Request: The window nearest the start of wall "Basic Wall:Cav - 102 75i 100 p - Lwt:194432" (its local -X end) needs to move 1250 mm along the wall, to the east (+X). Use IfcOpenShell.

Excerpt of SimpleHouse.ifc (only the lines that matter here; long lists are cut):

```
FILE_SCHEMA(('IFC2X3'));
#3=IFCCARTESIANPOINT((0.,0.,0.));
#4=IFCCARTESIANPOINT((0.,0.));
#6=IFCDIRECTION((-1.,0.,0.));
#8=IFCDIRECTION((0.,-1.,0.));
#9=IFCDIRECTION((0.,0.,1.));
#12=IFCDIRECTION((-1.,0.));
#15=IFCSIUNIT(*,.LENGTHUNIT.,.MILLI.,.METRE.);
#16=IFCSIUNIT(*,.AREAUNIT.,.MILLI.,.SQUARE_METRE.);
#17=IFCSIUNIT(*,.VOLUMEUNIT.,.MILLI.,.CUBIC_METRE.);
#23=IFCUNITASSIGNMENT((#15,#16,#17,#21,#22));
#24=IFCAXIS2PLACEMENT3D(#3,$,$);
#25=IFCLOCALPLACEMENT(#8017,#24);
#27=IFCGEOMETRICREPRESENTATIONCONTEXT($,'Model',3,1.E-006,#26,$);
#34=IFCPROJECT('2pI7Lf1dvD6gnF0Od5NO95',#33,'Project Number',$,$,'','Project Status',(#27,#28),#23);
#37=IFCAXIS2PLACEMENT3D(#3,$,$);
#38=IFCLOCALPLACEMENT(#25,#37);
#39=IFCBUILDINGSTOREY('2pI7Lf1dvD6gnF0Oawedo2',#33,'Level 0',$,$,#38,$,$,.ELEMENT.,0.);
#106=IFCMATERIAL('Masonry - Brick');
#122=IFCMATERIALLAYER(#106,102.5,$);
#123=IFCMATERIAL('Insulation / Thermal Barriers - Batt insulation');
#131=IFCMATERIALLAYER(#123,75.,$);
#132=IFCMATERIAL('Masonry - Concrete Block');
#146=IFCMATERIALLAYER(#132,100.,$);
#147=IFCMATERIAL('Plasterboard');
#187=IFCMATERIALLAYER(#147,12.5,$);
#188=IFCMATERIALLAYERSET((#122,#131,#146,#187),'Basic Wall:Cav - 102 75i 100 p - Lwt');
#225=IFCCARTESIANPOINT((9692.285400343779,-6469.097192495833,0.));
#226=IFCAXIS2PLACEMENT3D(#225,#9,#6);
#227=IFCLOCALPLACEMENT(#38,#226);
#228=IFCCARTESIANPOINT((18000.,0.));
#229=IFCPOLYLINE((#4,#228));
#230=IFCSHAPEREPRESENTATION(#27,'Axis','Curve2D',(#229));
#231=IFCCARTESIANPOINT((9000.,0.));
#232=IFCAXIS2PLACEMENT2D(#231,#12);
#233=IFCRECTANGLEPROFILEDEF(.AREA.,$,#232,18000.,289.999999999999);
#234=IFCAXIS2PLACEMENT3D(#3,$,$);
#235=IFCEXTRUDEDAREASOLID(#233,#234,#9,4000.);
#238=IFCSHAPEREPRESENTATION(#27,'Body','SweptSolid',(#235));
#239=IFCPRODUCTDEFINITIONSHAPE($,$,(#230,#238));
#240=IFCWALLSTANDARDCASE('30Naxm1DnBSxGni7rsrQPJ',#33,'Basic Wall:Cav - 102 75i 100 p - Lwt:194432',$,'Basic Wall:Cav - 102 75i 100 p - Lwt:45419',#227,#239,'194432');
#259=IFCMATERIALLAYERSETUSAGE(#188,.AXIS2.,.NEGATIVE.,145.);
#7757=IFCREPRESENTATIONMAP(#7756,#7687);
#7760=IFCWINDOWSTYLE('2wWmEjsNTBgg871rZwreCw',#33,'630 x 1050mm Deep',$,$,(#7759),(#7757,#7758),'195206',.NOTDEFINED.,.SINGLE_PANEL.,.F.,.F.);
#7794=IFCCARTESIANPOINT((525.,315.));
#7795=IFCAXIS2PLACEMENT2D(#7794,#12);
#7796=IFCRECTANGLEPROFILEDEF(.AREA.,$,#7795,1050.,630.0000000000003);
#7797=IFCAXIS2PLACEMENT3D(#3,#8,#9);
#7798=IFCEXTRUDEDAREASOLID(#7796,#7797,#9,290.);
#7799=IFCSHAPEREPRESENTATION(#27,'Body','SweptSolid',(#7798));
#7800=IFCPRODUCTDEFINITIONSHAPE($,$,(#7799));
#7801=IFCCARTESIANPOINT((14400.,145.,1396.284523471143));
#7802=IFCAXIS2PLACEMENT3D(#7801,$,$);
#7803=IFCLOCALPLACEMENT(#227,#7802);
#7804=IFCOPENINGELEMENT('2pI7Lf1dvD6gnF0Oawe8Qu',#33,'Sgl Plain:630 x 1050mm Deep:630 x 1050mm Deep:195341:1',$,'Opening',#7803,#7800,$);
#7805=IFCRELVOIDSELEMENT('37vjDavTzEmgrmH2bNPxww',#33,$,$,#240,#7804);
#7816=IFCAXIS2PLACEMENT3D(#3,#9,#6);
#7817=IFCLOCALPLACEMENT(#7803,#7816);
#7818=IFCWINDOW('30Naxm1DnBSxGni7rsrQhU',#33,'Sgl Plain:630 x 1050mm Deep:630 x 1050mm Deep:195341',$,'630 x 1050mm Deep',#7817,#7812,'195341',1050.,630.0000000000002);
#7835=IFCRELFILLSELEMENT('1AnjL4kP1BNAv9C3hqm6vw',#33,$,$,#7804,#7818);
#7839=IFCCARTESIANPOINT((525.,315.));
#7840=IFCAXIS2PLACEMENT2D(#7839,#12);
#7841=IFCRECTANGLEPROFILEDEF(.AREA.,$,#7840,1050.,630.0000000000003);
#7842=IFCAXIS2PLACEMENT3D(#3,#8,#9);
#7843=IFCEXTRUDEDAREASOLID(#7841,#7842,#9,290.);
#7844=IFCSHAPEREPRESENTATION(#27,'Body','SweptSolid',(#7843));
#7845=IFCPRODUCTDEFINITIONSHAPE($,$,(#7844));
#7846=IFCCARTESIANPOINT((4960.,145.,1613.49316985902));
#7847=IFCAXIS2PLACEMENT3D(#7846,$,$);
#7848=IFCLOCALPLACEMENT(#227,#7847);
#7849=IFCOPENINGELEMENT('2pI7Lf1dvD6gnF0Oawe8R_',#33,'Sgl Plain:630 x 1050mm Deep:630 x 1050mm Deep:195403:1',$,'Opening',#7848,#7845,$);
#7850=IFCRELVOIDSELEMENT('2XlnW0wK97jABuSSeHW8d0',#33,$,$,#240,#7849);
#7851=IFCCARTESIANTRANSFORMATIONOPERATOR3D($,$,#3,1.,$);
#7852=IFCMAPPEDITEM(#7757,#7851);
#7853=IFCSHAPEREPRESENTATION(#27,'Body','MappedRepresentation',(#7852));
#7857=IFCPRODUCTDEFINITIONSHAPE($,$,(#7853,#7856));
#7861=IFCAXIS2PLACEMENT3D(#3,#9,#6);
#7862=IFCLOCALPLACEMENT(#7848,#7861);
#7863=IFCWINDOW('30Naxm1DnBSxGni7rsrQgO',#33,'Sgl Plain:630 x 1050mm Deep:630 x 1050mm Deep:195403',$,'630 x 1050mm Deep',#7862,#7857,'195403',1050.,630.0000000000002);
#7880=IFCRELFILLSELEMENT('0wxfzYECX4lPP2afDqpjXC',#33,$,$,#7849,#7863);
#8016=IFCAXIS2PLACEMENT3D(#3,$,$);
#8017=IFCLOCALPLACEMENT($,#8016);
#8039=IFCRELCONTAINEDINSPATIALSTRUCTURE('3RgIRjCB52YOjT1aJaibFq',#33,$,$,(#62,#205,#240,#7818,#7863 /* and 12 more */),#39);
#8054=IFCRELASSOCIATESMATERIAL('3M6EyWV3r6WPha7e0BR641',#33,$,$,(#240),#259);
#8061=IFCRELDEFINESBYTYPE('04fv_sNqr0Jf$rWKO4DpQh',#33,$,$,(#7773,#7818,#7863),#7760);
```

```python
import ifcopenshell
import ifcopenshell.api.geometry
import ifcopenshell.util.placement
import ifcopenshell.util.unit

model = ifcopenshell.open("SimpleHouse.ifc")
unit_scale = ifcopenshell.util.unit.calculate_unit_scale(model)

window = model.by_guid("30Naxm1DnBSxGni7rsrQgO")
opening = window.FillsVoids[0].RelatingOpeningElement
wall = opening.VoidsElements[0].RelatingBuildingElement

wall_matrix = ifcopenshell.util.placement.get_local_placement(wall.ObjectPlacement)
shift = wall_matrix[:3, 0] * -1.25 / unit_scale
before = ifcopenshell.util.placement.get_local_placement(window.ObjectPlacement)[:3, 3].copy()

# The window is placed relative to its opening, so it follows when the opening moves.
matrix = ifcopenshell.util.placement.get_local_placement(opening.ObjectPlacement)
matrix[:3, 3] += shift
ifcopenshell.api.geometry.edit_object_placement(
    model, product=opening, matrix=matrix, is_si=False, should_transform_children=True
)

after = ifcopenshell.util.placement.get_local_placement(window.ObjectPlacement)[:3, 3]
print("window moved by", (after - before).round(3) + 0.0)

model.write("SimpleHouse_updated.ifc")
```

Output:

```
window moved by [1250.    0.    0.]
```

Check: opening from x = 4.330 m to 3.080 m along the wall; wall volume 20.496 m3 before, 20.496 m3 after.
